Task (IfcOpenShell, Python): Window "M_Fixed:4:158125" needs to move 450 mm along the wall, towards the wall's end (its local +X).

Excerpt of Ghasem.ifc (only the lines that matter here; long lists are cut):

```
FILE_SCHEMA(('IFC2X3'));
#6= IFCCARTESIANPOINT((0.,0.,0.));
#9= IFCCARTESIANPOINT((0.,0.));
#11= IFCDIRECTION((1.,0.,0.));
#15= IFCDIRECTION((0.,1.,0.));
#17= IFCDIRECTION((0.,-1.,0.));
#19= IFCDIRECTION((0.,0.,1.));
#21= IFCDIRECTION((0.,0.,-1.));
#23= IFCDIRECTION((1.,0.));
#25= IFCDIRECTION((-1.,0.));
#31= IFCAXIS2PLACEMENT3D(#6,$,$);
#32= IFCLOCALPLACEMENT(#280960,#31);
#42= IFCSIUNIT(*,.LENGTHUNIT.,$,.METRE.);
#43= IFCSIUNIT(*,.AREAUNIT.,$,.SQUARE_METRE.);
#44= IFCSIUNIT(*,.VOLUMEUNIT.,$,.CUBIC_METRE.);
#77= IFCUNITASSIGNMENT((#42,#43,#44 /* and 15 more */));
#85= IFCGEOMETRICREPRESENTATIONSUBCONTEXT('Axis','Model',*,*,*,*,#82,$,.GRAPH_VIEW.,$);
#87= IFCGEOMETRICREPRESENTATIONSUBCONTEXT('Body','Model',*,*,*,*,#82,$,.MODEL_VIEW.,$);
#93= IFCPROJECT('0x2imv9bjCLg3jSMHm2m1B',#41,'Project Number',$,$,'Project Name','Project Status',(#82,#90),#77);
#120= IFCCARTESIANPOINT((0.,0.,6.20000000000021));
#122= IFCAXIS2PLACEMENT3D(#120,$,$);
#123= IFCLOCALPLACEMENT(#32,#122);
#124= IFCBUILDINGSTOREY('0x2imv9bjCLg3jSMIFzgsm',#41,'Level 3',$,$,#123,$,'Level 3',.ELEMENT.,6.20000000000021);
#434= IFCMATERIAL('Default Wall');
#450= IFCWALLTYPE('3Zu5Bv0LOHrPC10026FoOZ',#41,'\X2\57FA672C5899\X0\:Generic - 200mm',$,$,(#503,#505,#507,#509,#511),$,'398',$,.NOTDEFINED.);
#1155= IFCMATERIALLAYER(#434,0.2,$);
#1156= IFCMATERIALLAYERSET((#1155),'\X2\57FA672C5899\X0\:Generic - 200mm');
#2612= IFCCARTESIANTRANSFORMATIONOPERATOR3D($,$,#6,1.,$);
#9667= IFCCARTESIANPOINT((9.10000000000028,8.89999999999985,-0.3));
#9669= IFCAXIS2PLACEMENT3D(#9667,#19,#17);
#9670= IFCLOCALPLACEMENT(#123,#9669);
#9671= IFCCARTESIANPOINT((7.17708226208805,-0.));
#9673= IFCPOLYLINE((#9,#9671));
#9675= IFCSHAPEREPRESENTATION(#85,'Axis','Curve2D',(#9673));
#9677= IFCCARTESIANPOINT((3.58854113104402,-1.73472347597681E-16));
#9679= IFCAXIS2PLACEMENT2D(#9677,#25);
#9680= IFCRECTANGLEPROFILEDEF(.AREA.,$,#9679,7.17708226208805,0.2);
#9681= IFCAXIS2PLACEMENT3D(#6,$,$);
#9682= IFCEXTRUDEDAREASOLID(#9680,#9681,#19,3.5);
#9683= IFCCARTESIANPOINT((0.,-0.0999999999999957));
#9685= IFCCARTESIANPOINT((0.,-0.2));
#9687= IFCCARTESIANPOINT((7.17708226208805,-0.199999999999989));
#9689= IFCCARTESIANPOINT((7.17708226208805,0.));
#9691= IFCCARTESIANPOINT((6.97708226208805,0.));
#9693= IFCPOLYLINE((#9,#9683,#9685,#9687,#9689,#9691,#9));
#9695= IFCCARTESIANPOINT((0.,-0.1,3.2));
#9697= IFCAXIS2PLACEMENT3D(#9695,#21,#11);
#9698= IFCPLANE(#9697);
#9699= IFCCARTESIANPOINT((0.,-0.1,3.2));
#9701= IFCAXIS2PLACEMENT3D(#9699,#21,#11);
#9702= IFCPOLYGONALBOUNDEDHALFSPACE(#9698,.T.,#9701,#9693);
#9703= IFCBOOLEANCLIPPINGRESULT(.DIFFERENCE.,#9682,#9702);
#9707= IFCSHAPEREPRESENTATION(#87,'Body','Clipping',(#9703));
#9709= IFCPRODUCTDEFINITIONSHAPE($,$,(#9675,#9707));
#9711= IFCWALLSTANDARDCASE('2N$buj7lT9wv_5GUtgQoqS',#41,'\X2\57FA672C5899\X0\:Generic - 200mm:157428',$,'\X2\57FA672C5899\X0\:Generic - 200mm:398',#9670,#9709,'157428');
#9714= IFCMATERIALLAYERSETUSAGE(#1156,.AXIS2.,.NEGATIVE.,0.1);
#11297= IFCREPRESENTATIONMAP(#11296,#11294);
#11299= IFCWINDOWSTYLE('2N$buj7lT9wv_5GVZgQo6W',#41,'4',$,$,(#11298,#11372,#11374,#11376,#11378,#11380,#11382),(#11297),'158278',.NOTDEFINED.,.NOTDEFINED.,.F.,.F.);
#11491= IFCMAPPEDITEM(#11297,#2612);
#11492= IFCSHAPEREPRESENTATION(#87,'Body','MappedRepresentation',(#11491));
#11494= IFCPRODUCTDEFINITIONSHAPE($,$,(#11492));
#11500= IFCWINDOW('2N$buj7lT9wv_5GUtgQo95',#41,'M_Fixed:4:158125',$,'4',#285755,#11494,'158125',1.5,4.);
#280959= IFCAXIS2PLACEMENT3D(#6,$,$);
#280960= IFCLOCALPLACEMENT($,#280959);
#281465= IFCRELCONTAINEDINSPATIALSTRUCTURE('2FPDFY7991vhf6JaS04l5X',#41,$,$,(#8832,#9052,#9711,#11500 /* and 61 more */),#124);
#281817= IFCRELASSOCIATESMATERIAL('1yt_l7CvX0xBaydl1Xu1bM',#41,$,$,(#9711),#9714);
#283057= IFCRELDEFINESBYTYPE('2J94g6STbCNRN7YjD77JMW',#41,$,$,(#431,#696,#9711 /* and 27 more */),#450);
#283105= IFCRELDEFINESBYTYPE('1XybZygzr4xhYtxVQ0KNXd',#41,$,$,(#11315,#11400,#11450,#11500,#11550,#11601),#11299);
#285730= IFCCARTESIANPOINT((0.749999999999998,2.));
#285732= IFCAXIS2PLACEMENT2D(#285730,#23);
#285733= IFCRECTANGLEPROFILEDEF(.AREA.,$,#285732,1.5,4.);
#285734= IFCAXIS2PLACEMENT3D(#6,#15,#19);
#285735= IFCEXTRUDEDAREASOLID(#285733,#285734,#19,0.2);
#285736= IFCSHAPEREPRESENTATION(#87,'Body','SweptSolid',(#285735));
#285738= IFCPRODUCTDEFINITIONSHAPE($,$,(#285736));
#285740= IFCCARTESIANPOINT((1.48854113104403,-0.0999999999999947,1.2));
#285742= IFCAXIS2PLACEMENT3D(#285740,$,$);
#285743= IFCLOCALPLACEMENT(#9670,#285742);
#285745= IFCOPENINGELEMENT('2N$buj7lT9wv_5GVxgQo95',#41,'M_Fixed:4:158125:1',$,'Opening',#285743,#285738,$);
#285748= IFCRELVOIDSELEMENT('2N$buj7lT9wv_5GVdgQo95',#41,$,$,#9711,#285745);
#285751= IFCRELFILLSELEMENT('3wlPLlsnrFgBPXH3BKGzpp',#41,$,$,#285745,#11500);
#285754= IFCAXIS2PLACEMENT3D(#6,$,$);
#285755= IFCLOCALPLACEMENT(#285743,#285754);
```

```python
import ifcopenshell
import ifcopenshell.api.geometry
import ifcopenshell.util.placement
import ifcopenshell.util.unit

model = ifcopenshell.open("Ghasem.ifc")
unit_scale = ifcopenshell.util.unit.calculate_unit_scale(model)

window = model.by_guid("2N$buj7lT9wv_5GUtgQo95")
opening = window.FillsVoids[0].RelatingOpeningElement
wall = opening.VoidsElements[0].RelatingBuildingElement

wall_matrix = ifcopenshell.util.placement.get_local_placement(wall.ObjectPlacement)
shift = wall_matrix[:3, 0] * 0.45 / unit_scale
before = ifcopenshell.util.placement.get_local_placement(window.ObjectPlacement)[:3, 3].copy()

# The window is placed relative to its opening, so it follows when the opening moves.
matrix = ifcopenshell.util.placement.get_local_placement(opening.ObjectPlacement)
matrix[:3, 3] += shift
ifcopenshell.api.geometry.edit_object_placement(
    model, product=opening, matrix=matrix, is_si=False, should_transform_children=True
)

after = ifcopenshell.util.placement.get_local_placement(window.ObjectPlacement)[:3, 3]
print("window moved by", (after - before).round(3) + 0.0)

model.write("Ghasem_rev.ifc")
```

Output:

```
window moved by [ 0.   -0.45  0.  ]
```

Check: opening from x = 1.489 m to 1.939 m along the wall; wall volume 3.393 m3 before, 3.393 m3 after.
